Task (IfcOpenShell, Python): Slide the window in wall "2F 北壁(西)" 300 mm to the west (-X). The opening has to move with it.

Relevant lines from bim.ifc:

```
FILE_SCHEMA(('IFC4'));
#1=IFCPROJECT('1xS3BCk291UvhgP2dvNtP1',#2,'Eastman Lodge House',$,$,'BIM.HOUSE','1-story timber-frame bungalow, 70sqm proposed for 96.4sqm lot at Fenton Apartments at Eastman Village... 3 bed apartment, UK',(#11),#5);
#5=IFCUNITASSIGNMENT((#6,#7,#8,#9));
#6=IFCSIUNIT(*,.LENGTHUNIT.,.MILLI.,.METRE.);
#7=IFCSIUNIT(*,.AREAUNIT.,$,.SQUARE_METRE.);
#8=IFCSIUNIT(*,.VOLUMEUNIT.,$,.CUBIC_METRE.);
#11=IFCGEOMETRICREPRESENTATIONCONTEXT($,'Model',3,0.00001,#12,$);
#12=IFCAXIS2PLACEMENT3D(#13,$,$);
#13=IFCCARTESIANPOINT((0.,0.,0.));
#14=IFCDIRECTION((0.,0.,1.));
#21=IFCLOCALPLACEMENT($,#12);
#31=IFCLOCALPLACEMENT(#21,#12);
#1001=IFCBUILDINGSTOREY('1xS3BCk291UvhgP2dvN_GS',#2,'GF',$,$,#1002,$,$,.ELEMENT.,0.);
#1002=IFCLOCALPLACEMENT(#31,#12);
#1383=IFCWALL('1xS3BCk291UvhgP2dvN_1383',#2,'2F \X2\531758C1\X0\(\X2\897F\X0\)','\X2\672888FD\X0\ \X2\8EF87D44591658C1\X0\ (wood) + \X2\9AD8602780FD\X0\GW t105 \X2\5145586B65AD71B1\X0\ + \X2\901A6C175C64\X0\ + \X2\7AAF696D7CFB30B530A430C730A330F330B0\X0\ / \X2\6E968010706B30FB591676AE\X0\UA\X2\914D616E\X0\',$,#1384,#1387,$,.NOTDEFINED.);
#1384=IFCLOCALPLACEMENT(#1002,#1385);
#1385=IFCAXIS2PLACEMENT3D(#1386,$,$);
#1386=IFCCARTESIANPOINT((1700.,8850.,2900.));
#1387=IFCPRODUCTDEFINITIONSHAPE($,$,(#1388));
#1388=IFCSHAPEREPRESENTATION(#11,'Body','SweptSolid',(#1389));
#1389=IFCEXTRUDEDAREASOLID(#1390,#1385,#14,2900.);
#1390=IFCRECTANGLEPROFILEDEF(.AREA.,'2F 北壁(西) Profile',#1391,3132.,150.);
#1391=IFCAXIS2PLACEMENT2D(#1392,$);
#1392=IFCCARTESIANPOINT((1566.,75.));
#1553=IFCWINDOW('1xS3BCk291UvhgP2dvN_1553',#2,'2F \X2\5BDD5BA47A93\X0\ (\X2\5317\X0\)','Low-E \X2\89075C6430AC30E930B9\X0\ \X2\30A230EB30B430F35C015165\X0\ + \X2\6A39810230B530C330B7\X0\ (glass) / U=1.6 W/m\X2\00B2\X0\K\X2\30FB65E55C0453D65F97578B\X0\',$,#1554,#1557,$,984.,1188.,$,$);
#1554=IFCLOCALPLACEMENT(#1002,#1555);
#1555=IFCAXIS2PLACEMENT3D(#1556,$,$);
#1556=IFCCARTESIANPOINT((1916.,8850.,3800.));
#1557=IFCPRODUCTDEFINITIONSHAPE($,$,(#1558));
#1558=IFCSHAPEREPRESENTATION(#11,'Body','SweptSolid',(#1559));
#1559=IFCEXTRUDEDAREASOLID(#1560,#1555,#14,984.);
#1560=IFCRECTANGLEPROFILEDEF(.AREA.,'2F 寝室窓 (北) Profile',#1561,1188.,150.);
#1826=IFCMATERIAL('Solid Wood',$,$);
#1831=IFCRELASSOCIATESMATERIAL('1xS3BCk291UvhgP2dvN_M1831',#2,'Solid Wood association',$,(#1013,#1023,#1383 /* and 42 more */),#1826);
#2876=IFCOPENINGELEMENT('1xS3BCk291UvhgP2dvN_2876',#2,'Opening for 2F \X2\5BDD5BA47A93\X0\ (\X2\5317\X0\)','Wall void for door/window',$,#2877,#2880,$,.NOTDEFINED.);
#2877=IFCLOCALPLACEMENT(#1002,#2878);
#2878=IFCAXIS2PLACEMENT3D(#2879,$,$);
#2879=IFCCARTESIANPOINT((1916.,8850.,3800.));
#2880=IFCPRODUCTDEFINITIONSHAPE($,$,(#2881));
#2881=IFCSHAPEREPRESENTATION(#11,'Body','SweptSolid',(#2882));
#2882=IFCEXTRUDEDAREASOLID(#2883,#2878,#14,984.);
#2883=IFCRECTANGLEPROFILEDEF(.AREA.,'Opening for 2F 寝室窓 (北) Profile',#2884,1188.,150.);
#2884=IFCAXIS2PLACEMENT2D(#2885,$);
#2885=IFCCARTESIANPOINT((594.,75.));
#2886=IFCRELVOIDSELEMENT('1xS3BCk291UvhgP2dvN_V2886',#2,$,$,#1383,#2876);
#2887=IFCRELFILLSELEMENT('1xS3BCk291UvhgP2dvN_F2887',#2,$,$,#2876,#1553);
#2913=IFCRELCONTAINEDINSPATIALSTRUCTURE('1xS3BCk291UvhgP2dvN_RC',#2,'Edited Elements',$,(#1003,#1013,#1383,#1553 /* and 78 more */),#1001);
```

```python
import ifcopenshell
import ifcopenshell.api.geometry
import ifcopenshell.util.placement
import ifcopenshell.util.unit

model = ifcopenshell.open("bim.ifc")
unit_scale = ifcopenshell.util.unit.calculate_unit_scale(model)

window = model.by_guid("1xS3BCk291UvhgP2dvN_1553")
opening = window.FillsVoids[0].RelatingOpeningElement
wall = opening.VoidsElements[0].RelatingBuildingElement

wall_matrix = ifcopenshell.util.placement.get_local_placement(wall.ObjectPlacement)
shift = wall_matrix[:3, 0] * -0.3 / unit_scale
before = ifcopenshell.util.placement.get_local_placement(window.ObjectPlacement)[:3, 3].copy()

# The window is not placed relative to its opening, so move both.
for product in (opening, window):
    matrix = ifcopenshell.util.placement.get_local_placement(product.ObjectPlacement)
    matrix[:3, 3] += shift
    ifcopenshell.api.geometry.edit_object_placement(model, product=product, matrix=matrix, is_si=False)

after = ifcopenshell.util.placement.get_local_placement(window.ObjectPlacement)[:3, 3]
print("window moved by", (after - before).round(3) + 0.0)

model.write("bim-out.ifc")
```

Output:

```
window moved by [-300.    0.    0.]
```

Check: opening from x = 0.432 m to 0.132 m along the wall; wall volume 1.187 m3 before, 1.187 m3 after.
